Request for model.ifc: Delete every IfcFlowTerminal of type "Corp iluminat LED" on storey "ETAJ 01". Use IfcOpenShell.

First a look at what the model holds.

```python
import ifcopenshell
import ifcopenshell.util.element

model = ifcopenshell.open("model.ifc")
print(model.schema)
storey = next(s for s in model.by_type("IfcBuildingStorey") if s.Name == "ETAJ 01")
terminals = [e for e in ifcopenshell.util.element.get_decomposition(storey) if e.is_a("IfcFlowTerminal")]
seen = {}
for e in terminals:
    element_type = ifcopenshell.util.element.get_type(e)
    name = element_type.Name if element_type not in (None, e) else None
    seen[name] = seen.get(name, 0) + 1
for name, count in sorted(seen.items(), key=str):
    print(count, "x", name)
```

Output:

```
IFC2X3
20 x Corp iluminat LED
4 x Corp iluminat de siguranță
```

```python
import ifcopenshell
import ifcopenshell.api.root
import ifcopenshell.util.element

model = ifcopenshell.open("model.ifc")

storey = next(s for s in model.by_type("IfcBuildingStorey") if s.Name == "ETAJ 01")
terminals = [e for e in ifcopenshell.util.element.get_decomposition(storey) if e.is_a("IfcFlowTerminal")]
targets = [e for e in terminals if (t := ifcopenshell.util.element.get_type(e)) not in (None, e) and t.Name == "Corp iluminat LED"]

for e in targets:
    ifcopenshell.api.root.remove_product(model, product=e)
print(len(targets), "removed")

model.write("model-out.ifc")
```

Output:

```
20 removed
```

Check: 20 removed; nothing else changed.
